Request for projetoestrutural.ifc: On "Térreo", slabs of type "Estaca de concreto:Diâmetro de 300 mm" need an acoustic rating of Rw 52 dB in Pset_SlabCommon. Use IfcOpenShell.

First a look at what the model holds.

```python
import ifcopenshell
import ifcopenshell.util.element

model = ifcopenshell.open("projetoestrutural.ifc")
print(model.schema)
storey = next(s for s in model.by_type("IfcBuildingStorey") if s.Name == "Térreo")
slabs = [e for e in ifcopenshell.util.element.get_decomposition(storey) if e.is_a("IfcSlab")]
seen = {}
for e in slabs:
    element_type = ifcopenshell.util.element.get_type(e)
    key = (element_type.Name if element_type != e and element_type else None, ifcopenshell.util.element.get_pset(e, "Pset_SlabCommon", "AcousticRating"))
    seen[key] = seen.get(key, 0) + 1
for (name, value), count in sorted(seen.items(), key=str):
    print(count, "x", name, "|", value)
```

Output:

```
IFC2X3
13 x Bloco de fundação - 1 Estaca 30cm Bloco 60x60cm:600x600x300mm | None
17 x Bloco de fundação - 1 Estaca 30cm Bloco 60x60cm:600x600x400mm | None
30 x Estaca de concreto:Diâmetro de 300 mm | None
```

```python
import ifcopenshell
import ifcopenshell.api.pset
import ifcopenshell.util.element

model = ifcopenshell.open("projetoestrutural.ifc")

storey = next(s for s in model.by_type("IfcBuildingStorey") if s.Name == "Térreo")
slabs = [e for e in ifcopenshell.util.element.get_decomposition(storey) if e.is_a("IfcSlab")]

count = 0
for e in slabs:
    element_type = ifcopenshell.util.element.get_type(e)
    if element_type in (None, e) or element_type.Name != "Estaca de concreto:Diâmetro de 300 mm":
        continue
    # add_pset returns the element's existing set when there is one.
    pset = ifcopenshell.api.pset.add_pset(model, product=e, name="Pset_SlabCommon")
    ifcopenshell.api.pset.edit_pset(model, pset=pset, properties={"AcousticRating": "Rw 52 dB"})
    count += 1

print(count, "slabs updated")

model.write("projetoestrutural_rev.ifc")
```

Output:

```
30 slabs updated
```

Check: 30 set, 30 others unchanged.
